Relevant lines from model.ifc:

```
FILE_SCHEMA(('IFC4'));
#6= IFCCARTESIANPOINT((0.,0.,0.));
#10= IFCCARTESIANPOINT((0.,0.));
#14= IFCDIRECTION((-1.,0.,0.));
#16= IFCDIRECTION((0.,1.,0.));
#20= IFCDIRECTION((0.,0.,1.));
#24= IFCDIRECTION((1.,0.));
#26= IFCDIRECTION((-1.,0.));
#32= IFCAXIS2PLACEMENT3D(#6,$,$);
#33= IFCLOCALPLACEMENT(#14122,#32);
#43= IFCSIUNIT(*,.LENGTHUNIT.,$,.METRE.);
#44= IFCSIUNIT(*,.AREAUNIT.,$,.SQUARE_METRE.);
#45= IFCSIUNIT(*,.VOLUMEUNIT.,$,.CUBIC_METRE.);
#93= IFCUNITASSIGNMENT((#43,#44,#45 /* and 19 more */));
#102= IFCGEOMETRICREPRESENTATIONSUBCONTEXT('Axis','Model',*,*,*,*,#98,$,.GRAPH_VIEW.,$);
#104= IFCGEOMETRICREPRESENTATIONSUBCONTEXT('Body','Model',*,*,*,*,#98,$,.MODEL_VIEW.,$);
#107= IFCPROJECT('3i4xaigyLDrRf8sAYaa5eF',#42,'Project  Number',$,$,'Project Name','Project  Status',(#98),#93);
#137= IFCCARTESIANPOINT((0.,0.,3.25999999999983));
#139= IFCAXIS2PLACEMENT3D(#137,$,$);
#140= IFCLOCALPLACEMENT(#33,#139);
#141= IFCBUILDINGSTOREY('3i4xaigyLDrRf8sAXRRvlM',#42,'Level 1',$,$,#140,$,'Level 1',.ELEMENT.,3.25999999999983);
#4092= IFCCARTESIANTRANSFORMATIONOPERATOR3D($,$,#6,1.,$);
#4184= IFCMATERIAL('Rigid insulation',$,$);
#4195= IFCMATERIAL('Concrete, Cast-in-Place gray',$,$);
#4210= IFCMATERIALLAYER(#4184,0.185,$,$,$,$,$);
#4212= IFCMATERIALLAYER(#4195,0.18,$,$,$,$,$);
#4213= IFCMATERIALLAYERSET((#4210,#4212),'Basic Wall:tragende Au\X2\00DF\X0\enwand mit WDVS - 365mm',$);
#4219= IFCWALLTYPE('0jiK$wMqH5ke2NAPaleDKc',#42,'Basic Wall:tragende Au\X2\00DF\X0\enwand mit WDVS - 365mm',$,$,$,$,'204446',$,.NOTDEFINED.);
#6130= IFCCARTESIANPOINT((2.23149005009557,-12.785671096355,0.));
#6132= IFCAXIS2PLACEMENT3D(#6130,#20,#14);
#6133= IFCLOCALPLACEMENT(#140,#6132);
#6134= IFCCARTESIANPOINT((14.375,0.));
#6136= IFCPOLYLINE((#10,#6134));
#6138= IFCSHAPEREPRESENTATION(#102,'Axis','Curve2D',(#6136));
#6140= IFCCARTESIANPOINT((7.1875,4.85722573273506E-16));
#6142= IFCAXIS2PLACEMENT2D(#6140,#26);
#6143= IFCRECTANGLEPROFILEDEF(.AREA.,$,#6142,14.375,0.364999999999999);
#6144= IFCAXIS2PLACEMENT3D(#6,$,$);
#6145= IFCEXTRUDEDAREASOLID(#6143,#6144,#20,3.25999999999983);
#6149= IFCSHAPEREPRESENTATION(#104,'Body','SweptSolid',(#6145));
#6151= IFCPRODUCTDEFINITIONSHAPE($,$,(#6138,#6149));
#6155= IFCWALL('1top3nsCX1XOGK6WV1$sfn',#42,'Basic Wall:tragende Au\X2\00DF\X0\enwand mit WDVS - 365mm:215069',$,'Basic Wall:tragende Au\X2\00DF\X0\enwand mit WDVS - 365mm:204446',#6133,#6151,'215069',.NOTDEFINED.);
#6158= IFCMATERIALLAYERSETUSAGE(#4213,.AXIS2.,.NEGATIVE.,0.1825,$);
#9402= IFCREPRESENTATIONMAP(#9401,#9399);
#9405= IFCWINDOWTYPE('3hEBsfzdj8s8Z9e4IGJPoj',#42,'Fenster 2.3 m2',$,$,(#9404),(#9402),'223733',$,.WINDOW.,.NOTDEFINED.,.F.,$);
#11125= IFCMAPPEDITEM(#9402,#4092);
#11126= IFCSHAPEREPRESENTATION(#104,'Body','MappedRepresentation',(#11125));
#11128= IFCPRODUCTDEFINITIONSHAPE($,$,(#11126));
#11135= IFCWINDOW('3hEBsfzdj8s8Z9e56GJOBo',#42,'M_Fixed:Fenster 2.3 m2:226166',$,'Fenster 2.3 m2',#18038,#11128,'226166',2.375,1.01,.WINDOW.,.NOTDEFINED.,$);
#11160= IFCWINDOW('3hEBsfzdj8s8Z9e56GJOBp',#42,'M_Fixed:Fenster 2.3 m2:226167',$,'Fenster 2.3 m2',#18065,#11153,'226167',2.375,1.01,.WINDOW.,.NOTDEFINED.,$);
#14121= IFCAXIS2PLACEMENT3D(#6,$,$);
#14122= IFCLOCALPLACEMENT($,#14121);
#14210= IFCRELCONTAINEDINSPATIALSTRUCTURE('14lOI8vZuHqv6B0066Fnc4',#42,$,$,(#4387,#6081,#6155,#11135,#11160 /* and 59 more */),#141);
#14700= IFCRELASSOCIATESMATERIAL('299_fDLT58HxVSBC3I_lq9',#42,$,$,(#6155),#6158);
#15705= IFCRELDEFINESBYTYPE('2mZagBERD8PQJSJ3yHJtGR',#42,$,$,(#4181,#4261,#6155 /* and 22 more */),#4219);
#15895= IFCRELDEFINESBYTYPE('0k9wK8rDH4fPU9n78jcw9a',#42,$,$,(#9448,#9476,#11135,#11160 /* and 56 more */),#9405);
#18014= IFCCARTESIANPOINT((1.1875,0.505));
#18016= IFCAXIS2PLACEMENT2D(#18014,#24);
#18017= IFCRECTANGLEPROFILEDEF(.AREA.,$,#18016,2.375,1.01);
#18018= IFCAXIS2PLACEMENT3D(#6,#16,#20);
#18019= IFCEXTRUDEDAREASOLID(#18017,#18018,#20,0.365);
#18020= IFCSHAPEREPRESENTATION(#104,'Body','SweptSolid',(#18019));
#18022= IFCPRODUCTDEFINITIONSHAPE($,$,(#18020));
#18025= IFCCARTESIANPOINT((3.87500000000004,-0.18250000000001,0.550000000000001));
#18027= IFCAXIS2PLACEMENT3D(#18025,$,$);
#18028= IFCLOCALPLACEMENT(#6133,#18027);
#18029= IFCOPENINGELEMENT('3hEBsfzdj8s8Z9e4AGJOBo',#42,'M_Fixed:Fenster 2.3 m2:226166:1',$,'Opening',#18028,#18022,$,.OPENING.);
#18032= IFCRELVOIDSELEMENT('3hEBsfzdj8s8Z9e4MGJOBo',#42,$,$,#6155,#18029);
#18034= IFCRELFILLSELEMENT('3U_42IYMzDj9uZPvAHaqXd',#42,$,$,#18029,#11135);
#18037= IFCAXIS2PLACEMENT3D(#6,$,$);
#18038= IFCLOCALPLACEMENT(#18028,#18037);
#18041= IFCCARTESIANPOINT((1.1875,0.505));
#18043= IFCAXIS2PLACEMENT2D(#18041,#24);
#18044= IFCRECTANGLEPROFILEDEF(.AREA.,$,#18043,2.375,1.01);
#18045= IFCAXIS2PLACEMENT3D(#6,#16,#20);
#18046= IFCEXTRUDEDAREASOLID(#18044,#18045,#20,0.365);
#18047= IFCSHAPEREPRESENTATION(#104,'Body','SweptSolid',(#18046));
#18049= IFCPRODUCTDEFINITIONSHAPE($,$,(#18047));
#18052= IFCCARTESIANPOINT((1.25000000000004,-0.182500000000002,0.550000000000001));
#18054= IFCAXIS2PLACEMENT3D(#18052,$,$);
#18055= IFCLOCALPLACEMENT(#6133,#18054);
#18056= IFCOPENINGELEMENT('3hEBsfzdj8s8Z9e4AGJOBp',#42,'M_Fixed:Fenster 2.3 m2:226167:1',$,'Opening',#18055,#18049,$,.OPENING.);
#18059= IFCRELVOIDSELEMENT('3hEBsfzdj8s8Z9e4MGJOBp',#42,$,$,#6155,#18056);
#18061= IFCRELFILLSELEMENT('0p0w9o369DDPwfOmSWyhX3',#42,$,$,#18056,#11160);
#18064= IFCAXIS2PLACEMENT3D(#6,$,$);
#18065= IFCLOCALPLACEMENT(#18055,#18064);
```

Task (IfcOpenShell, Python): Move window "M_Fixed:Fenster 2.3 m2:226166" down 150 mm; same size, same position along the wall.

```python
import numpy as np
import ifcopenshell
import ifcopenshell.api.geometry
import ifcopenshell.util.placement
import ifcopenshell.util.unit

model = ifcopenshell.open("model.ifc")
unit_scale = ifcopenshell.util.unit.calculate_unit_scale(model)

window = model.by_guid("3hEBsfzdj8s8Z9e56GJOBo")
opening = window.FillsVoids[0].RelatingOpeningElement
dz = -0.15

shift = np.array([0.0, 0.0, dz])
# The window is placed relative to its opening, so it follows when the opening moves.
matrix = ifcopenshell.util.placement.get_local_placement(opening.ObjectPlacement)
matrix[:3, 3] += shift
ifcopenshell.api.geometry.edit_object_placement(
    model, product=opening, matrix=matrix, is_si=False, should_transform_children=True
)

print(f"moved by {dz * unit_scale:+.3f} m")

model.write("model_updated.ifc")
```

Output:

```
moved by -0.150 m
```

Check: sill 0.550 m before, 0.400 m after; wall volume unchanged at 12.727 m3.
